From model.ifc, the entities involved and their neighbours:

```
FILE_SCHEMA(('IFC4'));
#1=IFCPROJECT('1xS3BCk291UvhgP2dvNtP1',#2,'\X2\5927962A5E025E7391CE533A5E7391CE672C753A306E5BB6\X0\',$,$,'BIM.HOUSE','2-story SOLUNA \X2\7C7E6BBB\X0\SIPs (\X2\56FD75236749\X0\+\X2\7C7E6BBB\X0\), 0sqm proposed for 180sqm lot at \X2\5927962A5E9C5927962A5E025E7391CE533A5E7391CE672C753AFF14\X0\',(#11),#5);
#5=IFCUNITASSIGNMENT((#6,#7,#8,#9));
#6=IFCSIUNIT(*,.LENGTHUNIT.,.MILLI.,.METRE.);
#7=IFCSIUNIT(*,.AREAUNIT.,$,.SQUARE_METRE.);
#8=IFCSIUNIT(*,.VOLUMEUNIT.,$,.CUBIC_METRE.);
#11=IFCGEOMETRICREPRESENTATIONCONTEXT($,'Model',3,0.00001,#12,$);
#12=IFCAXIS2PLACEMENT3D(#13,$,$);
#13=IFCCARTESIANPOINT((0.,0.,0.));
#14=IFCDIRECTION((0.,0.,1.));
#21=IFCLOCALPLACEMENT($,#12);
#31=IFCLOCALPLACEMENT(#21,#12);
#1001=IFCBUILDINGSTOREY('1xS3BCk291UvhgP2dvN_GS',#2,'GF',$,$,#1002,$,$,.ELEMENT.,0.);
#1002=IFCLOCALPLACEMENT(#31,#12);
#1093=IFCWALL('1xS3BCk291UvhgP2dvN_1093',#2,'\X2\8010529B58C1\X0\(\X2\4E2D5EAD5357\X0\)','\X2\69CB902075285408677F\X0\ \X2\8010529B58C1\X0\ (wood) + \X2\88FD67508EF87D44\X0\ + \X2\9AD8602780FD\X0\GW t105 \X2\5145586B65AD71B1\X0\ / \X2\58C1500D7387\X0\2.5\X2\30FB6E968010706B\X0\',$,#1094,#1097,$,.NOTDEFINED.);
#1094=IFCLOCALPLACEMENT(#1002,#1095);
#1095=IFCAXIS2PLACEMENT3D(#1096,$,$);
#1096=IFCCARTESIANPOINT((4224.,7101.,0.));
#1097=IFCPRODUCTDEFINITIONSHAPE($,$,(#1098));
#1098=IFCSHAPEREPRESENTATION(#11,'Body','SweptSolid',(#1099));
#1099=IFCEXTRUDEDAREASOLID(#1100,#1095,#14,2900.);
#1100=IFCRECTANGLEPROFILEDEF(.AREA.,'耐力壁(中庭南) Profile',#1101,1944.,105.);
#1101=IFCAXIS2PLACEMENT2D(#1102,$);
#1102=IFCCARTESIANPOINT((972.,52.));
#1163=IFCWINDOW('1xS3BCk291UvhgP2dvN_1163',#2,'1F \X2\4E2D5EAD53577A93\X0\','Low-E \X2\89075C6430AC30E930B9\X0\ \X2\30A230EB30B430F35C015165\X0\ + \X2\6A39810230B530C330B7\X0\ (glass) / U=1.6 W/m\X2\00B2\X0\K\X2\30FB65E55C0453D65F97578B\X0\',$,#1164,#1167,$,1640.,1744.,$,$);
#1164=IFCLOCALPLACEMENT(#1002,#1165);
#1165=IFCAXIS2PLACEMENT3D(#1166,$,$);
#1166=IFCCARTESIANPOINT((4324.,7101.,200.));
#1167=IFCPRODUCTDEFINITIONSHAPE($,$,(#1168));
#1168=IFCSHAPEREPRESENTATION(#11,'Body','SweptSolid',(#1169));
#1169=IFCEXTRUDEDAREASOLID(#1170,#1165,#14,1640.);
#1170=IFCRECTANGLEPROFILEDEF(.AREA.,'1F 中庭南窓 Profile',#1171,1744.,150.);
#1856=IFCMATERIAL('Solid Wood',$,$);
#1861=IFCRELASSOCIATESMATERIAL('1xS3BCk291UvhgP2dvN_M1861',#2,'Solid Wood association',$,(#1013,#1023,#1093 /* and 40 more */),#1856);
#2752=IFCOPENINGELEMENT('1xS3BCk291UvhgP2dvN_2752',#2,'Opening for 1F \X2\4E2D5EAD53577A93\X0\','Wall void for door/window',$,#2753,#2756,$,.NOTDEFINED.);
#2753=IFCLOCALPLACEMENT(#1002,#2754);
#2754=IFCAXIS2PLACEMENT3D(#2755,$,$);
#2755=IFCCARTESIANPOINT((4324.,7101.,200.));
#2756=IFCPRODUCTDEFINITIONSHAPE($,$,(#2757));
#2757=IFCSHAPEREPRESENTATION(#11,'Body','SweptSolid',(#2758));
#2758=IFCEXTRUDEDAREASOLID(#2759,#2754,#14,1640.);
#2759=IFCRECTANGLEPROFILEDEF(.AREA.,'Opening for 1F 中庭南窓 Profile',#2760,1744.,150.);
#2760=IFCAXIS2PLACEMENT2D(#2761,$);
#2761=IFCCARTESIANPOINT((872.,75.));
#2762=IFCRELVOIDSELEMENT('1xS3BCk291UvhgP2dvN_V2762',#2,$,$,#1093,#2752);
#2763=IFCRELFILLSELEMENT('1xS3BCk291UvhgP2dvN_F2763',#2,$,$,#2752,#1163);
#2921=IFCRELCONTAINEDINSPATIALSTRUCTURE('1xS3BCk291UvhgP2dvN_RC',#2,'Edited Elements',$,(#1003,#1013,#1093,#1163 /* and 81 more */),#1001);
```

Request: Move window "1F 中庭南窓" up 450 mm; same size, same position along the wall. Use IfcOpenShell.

```python
import numpy as np
import ifcopenshell
import ifcopenshell.api.geometry
import ifcopenshell.util.placement
import ifcopenshell.util.unit

model = ifcopenshell.open("model.ifc")
unit_scale = ifcopenshell.util.unit.calculate_unit_scale(model)

window = model.by_guid("1xS3BCk291UvhgP2dvN_1163")
opening = window.FillsVoids[0].RelatingOpeningElement
dz = 450.0

shift = np.array([0.0, 0.0, dz])
# The window is not placed relative to its opening, so move both.
for product in (opening, window):
    matrix = ifcopenshell.util.placement.get_local_placement(product.ObjectPlacement)
    matrix[:3, 3] += shift
    ifcopenshell.api.geometry.edit_object_placement(model, product=product, matrix=matrix, is_si=False)

print(f"moved by {dz * unit_scale:+.3f} m")

model.write("model_v2.ifc")
```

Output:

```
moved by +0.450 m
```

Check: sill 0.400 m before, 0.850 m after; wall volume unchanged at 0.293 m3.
